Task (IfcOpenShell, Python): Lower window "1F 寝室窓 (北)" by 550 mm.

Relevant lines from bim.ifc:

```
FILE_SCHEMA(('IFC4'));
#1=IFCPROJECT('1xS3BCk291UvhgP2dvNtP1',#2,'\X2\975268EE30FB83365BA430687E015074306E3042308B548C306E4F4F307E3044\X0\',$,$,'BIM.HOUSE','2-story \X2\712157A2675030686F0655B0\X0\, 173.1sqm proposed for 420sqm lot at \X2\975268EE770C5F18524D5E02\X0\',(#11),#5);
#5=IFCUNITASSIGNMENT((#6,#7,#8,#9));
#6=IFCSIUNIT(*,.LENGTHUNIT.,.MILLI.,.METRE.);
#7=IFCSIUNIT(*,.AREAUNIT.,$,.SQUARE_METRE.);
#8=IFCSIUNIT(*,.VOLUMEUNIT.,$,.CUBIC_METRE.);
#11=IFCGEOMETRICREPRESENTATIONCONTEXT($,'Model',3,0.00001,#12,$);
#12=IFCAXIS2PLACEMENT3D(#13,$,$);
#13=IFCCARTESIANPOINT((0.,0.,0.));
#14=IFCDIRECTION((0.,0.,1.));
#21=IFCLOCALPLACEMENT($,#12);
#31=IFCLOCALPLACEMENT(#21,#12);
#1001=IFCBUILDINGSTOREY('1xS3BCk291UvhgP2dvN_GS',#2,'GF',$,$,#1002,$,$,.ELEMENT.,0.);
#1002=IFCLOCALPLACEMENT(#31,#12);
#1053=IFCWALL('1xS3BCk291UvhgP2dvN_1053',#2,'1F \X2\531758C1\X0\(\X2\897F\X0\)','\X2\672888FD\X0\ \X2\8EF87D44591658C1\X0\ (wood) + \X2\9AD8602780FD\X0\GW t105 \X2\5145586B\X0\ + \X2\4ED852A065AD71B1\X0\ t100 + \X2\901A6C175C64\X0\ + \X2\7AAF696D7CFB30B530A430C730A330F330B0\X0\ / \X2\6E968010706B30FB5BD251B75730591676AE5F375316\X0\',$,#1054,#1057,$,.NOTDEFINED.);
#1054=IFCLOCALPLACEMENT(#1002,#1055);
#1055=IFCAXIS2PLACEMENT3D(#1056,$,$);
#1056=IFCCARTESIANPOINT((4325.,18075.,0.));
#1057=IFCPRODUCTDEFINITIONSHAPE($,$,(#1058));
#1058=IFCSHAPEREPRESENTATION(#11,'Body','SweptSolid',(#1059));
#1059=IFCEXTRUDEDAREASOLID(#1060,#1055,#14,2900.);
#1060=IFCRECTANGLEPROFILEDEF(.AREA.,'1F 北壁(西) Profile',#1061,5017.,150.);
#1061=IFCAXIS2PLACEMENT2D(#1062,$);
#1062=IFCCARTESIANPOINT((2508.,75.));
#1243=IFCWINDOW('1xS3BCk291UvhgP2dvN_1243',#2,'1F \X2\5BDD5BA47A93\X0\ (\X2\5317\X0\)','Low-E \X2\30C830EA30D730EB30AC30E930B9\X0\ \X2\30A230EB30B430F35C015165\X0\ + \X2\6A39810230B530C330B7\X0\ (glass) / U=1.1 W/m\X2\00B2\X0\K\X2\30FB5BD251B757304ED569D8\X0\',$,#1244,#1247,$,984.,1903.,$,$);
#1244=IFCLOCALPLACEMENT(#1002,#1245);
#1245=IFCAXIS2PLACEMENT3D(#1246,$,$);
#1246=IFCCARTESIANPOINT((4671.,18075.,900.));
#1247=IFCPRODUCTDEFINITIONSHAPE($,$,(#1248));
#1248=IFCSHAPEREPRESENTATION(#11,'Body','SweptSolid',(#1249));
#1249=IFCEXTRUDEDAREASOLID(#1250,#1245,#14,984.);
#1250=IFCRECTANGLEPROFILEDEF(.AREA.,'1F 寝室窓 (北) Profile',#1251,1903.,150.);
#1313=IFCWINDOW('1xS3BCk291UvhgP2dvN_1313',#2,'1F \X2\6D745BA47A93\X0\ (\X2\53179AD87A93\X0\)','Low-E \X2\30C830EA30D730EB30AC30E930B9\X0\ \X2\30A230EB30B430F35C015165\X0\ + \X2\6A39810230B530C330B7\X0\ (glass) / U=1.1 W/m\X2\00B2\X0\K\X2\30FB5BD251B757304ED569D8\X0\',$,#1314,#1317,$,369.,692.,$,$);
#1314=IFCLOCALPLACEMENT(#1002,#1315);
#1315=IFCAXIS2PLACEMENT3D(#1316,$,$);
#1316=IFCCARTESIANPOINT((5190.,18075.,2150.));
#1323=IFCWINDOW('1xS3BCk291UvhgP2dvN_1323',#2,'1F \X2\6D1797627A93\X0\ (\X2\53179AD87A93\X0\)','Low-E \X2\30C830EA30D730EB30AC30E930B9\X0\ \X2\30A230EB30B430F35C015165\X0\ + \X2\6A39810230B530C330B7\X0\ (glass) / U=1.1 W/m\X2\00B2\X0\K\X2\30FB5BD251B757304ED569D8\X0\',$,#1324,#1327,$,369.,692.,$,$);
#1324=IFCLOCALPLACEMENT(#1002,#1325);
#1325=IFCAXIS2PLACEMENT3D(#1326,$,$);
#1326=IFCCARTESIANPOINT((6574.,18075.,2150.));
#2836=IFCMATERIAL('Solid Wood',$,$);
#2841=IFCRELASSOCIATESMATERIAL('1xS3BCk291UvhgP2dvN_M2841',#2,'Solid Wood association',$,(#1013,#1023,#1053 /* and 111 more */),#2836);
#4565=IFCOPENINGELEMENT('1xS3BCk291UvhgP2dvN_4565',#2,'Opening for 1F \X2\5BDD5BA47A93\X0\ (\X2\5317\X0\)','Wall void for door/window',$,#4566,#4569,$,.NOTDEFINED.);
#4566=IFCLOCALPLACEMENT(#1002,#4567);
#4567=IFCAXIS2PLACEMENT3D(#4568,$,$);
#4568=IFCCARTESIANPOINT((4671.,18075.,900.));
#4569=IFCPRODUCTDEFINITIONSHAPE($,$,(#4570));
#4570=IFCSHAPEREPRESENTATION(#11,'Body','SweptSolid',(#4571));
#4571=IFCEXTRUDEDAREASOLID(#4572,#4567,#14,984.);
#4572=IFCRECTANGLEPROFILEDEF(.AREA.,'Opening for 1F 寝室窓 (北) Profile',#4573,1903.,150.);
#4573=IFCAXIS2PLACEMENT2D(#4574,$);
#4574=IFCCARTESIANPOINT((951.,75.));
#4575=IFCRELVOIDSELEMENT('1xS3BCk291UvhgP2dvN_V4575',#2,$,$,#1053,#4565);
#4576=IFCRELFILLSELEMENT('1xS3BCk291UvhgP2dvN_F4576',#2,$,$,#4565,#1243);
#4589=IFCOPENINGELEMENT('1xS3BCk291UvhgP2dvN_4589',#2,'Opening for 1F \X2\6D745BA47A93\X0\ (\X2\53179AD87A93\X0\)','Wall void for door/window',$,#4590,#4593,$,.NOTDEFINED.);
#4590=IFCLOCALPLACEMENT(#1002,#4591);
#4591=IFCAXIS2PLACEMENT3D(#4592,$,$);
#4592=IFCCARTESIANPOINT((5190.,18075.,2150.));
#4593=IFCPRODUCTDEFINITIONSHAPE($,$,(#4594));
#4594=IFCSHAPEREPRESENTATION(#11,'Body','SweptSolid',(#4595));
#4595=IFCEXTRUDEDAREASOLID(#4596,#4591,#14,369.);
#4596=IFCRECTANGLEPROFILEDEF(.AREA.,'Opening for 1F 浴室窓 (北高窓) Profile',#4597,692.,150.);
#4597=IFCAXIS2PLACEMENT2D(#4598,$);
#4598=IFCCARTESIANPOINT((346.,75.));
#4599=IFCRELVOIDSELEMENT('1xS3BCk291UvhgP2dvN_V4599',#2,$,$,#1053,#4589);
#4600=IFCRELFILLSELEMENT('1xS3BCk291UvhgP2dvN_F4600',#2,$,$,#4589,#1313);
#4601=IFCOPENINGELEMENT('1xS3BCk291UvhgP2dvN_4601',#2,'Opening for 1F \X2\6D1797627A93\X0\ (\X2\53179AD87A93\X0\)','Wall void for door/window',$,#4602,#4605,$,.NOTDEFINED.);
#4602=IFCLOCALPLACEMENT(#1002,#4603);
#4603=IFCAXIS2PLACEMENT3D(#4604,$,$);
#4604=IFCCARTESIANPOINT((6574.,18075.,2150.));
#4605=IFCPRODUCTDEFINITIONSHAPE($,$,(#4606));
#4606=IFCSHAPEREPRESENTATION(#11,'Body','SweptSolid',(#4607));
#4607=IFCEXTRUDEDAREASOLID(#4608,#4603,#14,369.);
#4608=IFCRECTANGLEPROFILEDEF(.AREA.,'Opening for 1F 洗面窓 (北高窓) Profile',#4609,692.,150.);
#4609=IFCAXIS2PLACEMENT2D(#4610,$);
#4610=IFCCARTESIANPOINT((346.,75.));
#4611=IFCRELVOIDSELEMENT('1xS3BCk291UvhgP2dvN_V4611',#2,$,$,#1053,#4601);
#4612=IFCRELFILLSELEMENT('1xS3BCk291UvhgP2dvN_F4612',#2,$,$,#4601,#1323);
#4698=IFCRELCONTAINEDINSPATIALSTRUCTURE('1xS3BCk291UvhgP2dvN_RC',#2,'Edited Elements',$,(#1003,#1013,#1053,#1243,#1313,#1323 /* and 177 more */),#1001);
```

```python
import numpy as np
import ifcopenshell
import ifcopenshell.api.geometry
import ifcopenshell.util.placement
import ifcopenshell.util.unit

model = ifcopenshell.open("bim.ifc")
unit_scale = ifcopenshell.util.unit.calculate_unit_scale(model)

window = model.by_guid("1xS3BCk291UvhgP2dvN_1243")
opening = window.FillsVoids[0].RelatingOpeningElement
dz = -550.0

shift = np.array([0.0, 0.0, dz])
# The window is not placed relative to its opening, so move both.
for product in (opening, window):
    matrix = ifcopenshell.util.placement.get_local_placement(product.ObjectPlacement)
    matrix[:3, 3] += shift
    ifcopenshell.api.geometry.edit_object_placement(model, product=product, matrix=matrix, is_si=False)

print(f"moved by {dz * unit_scale:+.3f} m")

model.write("bim_v2.ifc")
```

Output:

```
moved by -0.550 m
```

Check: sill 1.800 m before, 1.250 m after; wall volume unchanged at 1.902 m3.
